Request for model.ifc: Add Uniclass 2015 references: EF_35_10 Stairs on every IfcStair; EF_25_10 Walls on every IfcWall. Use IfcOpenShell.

First a look at what the model holds.

```python
import ifcopenshell

model = ifcopenshell.open("model.ifc")
print(model.schema)
print("classifications:", [c.Name for c in model.by_type("IfcClassification")])
for ifc_class in ("IfcDoor", "IfcRoof", "IfcStair", "IfcWall", "IfcWindow"):
    print(ifc_class, len(model.by_type(ifc_class)))
```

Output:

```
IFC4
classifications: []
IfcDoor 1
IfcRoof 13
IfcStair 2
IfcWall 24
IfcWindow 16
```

```python
import ifcopenshell
import ifcopenshell.api.classification

model = ifcopenshell.open("model.ifc")

system = ifcopenshell.api.classification.add_classification(model, classification="Uniclass 2015")

codes = {
    "IfcStair": ("EF_35_10", "Stairs"),
    "IfcWall": ("EF_25_10", "Walls"),
}
for ifc_class, (code, name) in codes.items():
    products = model.by_type(ifc_class)
    ifcopenshell.api.classification.add_reference(
        model, products=products, classification=system, identification=code, name=name
    )
    print(code, len(products))

model.write("model_v2.ifc")
```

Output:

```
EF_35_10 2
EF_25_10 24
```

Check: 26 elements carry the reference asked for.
